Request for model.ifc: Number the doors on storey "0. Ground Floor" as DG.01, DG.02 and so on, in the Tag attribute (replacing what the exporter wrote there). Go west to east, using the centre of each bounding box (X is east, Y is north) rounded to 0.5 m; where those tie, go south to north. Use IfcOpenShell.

First a look at what the model holds.

```python
import ifcopenshell
import ifcopenshell.util.element
import ifcopenshell.util.placement

model = ifcopenshell.open("model.ifc")
print(model.schema)
storey = next(s for s in model.by_type("IfcBuildingStorey") if s.Name == "0. Ground Floor")
doors = [e for e in ifcopenshell.util.element.get_decomposition(storey) if e.is_a("IfcDoor")]
for e in sorted(doors, key=lambda e: e.id()):
    origin = ifcopenshell.util.placement.get_local_placement(e.ObjectPlacement)[:3, 3]
    print(e.id(), e.Tag, e.Name, origin.round(2) + 0.0, sep=" | ")
```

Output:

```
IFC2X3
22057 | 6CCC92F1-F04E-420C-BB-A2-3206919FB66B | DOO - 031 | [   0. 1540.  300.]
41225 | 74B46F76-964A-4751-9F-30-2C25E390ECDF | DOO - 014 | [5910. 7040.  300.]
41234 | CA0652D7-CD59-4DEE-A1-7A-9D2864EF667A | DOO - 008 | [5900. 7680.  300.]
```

```python
import ifcopenshell
import ifcopenshell.geom
import ifcopenshell.util.element
import ifcopenshell.util.shape

model = ifcopenshell.open("model.ifc")
settings = ifcopenshell.geom.settings()
settings.set("use-world-coords", True)


def centre(element):
    shape = ifcopenshell.geom.create_shape(settings, element)
    return ifcopenshell.util.shape.get_bbox_centroid(shape.geometry)


storey = next(s for s in model.by_type("IfcBuildingStorey") if s.Name == "0. Ground Floor")
doors = [e for e in ifcopenshell.util.element.get_decomposition(storey) if e.is_a("IfcDoor")]

# Insertion points can sit at a corner or the storey origin, so sort by the geometry (in metres).
centres = {e: centre(e) for e in doors}
doors.sort(key=lambda e: (round(centres[e][0] / 0.5), centres[e][1]))

for i, e in enumerate(doors, start=1):
    number = f"DG.{i:02d}"
    e.Tag = number
    print(e.id(), number)

model.write("model-out.ifc")
```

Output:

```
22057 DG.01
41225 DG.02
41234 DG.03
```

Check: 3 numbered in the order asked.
